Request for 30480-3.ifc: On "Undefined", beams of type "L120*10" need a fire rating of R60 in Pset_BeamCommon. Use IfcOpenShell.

First a look at what the model holds.

```python
import ifcopenshell
import ifcopenshell.util.element

model = ifcopenshell.open("30480-3.ifc")
print(model.schema)
storey = next(s for s in model.by_type("IfcBuildingStorey") if s.Name == "Undefined")
beams = [e for e in ifcopenshell.util.element.get_decomposition(storey) if e.is_a("IfcBeam")]
seen = {}
for e in beams:
    element_type = ifcopenshell.util.element.get_type(e)
    key = (element_type.Name if element_type != e and element_type else None, ifcopenshell.util.element.get_pset(e, "Pset_BeamCommon", "FireRating"))
    seen[key] = seen.get(key, 0) + 1
for (name, value), count in sorted(seen.items(), key=str):
    print(count, "x", name, "|", value)
```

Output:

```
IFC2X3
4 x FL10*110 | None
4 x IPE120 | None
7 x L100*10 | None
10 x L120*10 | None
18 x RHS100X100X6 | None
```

```python
import ifcopenshell
import ifcopenshell.api.pset
import ifcopenshell.util.element

model = ifcopenshell.open("30480-3.ifc")

storey = next(s for s in model.by_type("IfcBuildingStorey") if s.Name == "Undefined")
beams = [e for e in ifcopenshell.util.element.get_decomposition(storey) if e.is_a("IfcBeam")]

count = 0
for e in beams:
    element_type = ifcopenshell.util.element.get_type(e)
    if element_type in (None, e) or element_type.Name != "L120*10":
        continue
    found = ifcopenshell.util.element.get_pset(e, "Pset_BeamCommon", should_inherit=False)
    if found:
        pset = model.by_id(found["id"])
        if len(ifcopenshell.util.element.get_elements_by_pset(pset)) > 1:
            pset = ifcopenshell.api.pset.unshare_pset(model, products=[e], pset=pset)[0]
    else:
        pset = ifcopenshell.api.pset.add_pset(model, product=e, name="Pset_BeamCommon")
    ifcopenshell.api.pset.edit_pset(model, pset=pset, properties={"FireRating": "R60"})
    count += 1

print(count, "beams updated")

model.write("30480-3_rev.ifc")
```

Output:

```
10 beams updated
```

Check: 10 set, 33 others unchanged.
